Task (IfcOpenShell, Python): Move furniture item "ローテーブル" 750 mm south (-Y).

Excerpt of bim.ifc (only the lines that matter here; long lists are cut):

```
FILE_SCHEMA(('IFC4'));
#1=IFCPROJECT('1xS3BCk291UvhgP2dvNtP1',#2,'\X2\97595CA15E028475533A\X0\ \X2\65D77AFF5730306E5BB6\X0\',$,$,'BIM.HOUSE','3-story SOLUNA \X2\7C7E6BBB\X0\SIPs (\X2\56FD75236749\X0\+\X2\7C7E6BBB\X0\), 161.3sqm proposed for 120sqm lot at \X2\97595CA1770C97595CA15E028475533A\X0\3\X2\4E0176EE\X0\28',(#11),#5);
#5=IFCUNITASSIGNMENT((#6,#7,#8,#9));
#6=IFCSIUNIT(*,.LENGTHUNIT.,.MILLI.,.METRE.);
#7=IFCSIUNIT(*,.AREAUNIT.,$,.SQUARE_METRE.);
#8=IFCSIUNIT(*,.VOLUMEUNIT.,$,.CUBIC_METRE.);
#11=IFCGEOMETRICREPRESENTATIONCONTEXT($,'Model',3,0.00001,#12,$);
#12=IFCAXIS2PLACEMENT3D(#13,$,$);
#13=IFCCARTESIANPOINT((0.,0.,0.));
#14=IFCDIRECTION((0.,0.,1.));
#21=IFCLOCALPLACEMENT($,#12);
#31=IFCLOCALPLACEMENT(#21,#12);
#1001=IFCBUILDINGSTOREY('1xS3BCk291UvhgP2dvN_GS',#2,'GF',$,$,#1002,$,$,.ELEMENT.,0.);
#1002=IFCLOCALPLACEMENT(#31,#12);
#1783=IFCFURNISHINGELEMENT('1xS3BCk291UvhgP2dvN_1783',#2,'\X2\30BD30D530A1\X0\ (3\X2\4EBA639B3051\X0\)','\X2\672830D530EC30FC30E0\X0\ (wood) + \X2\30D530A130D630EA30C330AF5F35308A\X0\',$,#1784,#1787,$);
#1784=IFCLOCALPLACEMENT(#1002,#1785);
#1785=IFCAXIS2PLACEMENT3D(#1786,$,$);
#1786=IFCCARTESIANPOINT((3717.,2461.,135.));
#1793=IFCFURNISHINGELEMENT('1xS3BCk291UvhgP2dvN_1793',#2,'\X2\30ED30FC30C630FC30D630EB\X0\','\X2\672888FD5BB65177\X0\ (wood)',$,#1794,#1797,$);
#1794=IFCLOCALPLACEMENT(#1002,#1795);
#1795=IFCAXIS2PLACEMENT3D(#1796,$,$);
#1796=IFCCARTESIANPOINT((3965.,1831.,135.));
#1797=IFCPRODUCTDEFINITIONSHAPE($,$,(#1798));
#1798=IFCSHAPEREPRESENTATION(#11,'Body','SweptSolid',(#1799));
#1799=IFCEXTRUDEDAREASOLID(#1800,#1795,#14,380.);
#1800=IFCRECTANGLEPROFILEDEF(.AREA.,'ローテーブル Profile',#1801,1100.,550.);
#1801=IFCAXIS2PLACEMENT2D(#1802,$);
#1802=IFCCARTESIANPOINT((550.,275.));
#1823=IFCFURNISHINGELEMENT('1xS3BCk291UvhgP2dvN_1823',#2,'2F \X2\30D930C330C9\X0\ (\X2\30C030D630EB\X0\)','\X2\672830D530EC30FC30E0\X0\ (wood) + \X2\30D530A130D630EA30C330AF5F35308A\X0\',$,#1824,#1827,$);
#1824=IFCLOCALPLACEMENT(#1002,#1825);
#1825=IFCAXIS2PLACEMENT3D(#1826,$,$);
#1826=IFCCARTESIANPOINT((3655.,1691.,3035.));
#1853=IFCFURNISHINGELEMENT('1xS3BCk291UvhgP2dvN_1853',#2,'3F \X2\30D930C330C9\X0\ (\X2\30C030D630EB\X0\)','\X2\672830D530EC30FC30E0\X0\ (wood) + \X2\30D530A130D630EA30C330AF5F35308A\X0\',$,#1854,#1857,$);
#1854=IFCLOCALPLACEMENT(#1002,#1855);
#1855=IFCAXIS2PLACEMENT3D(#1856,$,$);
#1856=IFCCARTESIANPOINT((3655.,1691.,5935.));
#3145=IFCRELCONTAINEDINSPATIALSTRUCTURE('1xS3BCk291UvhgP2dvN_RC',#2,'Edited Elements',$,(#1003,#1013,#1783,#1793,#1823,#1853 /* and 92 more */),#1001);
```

```python
import ifcopenshell
import ifcopenshell.api.geometry
import ifcopenshell.util.placement
import ifcopenshell.util.unit

model = ifcopenshell.open("bim.ifc")
unit_scale = ifcopenshell.util.unit.calculate_unit_scale(model)

item = model.by_id(1793)
matrix = ifcopenshell.util.placement.get_local_placement(item.ObjectPlacement)
matrix[1, 3] -= 0.75 / unit_scale
ifcopenshell.api.geometry.edit_object_placement(model, product=item, matrix=matrix, is_si=False)

print(ifcopenshell.util.placement.get_local_placement(item.ObjectPlacement).round(3) + 0.0)

model.write("bim-out.ifc")
```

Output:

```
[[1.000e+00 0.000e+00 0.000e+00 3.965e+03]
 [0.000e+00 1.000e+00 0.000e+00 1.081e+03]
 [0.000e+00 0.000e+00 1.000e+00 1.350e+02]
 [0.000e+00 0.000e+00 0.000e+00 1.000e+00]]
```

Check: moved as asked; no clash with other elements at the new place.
